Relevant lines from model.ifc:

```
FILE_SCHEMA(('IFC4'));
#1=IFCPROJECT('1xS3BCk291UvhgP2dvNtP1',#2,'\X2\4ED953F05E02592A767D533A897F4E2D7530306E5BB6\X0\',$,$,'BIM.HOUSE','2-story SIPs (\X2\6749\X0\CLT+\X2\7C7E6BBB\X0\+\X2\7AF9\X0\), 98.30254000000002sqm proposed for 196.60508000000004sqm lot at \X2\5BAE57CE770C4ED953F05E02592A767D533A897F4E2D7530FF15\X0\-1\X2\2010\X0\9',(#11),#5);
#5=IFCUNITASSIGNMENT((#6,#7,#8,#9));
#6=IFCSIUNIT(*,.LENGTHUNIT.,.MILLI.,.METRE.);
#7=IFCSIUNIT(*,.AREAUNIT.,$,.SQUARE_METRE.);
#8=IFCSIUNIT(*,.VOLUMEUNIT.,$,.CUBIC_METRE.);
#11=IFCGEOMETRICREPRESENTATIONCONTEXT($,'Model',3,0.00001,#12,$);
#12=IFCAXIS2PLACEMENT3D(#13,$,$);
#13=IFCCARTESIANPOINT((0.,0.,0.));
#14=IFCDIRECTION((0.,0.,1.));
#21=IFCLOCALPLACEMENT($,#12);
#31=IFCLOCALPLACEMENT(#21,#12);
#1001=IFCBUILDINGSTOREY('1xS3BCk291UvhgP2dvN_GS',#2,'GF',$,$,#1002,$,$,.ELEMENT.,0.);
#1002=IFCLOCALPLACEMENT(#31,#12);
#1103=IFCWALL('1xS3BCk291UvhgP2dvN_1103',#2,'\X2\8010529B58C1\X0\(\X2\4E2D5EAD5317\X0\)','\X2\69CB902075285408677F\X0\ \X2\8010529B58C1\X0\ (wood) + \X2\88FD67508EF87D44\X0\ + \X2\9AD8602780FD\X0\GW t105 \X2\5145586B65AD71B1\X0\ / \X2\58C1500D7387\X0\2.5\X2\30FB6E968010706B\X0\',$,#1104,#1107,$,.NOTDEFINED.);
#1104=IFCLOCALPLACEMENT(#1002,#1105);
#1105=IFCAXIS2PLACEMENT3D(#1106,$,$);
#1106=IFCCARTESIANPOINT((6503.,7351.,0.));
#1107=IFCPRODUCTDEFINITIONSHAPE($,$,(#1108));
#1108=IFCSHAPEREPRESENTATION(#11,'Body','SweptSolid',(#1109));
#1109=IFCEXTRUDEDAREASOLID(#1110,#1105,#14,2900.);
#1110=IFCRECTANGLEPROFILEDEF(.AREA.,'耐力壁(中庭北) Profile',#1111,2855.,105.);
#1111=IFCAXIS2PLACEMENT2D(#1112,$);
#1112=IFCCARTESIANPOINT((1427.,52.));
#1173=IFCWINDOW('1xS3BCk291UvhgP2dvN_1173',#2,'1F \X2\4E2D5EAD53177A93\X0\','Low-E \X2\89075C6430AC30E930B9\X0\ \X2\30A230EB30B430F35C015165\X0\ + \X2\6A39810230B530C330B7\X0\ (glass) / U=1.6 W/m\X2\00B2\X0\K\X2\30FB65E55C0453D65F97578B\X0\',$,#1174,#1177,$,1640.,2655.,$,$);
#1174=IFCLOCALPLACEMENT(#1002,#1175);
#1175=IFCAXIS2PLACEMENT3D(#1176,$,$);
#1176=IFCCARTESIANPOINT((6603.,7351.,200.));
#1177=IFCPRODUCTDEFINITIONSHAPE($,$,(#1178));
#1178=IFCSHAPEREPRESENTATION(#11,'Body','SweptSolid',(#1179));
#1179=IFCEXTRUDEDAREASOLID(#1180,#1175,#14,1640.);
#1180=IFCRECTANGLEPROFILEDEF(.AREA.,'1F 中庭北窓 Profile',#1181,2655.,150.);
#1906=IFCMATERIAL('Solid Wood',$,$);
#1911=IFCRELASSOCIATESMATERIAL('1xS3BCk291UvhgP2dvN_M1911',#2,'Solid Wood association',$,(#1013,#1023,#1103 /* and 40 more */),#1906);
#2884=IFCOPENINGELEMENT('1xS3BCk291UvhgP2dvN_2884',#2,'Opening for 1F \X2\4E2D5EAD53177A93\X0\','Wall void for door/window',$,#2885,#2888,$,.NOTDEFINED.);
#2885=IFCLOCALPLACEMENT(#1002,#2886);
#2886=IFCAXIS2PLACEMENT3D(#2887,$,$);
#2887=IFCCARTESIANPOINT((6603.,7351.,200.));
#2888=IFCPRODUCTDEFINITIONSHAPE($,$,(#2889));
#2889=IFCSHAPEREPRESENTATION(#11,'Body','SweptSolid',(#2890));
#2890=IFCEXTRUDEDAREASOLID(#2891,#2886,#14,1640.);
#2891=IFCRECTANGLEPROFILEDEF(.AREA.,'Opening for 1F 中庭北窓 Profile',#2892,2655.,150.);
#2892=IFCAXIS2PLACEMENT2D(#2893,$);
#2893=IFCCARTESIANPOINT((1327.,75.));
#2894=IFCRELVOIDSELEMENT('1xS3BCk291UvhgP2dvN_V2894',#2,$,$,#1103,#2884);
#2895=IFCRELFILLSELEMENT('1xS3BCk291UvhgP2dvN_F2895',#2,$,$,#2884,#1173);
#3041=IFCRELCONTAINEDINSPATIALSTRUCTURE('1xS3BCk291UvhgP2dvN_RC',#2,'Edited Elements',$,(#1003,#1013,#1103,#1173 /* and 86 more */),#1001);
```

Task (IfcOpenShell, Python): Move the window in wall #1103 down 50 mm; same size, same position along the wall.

```python
import numpy as np
import ifcopenshell
import ifcopenshell.api.geometry
import ifcopenshell.util.placement
import ifcopenshell.util.unit

model = ifcopenshell.open("model.ifc")
unit_scale = ifcopenshell.util.unit.calculate_unit_scale(model)

window = model.by_id(1173)
opening = window.FillsVoids[0].RelatingOpeningElement
dz = -50.0

shift = np.array([0.0, 0.0, dz])
# The window is not placed relative to its opening, so move both.
for product in (opening, window):
    matrix = ifcopenshell.util.placement.get_local_placement(product.ObjectPlacement)
    matrix[:3, 3] += shift
    ifcopenshell.api.geometry.edit_object_placement(model, product=product, matrix=matrix, is_si=False)

print(f"moved by {dz * unit_scale:+.3f} m")

model.write("model_v2.ifc")
```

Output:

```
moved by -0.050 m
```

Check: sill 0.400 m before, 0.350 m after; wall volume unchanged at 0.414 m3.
